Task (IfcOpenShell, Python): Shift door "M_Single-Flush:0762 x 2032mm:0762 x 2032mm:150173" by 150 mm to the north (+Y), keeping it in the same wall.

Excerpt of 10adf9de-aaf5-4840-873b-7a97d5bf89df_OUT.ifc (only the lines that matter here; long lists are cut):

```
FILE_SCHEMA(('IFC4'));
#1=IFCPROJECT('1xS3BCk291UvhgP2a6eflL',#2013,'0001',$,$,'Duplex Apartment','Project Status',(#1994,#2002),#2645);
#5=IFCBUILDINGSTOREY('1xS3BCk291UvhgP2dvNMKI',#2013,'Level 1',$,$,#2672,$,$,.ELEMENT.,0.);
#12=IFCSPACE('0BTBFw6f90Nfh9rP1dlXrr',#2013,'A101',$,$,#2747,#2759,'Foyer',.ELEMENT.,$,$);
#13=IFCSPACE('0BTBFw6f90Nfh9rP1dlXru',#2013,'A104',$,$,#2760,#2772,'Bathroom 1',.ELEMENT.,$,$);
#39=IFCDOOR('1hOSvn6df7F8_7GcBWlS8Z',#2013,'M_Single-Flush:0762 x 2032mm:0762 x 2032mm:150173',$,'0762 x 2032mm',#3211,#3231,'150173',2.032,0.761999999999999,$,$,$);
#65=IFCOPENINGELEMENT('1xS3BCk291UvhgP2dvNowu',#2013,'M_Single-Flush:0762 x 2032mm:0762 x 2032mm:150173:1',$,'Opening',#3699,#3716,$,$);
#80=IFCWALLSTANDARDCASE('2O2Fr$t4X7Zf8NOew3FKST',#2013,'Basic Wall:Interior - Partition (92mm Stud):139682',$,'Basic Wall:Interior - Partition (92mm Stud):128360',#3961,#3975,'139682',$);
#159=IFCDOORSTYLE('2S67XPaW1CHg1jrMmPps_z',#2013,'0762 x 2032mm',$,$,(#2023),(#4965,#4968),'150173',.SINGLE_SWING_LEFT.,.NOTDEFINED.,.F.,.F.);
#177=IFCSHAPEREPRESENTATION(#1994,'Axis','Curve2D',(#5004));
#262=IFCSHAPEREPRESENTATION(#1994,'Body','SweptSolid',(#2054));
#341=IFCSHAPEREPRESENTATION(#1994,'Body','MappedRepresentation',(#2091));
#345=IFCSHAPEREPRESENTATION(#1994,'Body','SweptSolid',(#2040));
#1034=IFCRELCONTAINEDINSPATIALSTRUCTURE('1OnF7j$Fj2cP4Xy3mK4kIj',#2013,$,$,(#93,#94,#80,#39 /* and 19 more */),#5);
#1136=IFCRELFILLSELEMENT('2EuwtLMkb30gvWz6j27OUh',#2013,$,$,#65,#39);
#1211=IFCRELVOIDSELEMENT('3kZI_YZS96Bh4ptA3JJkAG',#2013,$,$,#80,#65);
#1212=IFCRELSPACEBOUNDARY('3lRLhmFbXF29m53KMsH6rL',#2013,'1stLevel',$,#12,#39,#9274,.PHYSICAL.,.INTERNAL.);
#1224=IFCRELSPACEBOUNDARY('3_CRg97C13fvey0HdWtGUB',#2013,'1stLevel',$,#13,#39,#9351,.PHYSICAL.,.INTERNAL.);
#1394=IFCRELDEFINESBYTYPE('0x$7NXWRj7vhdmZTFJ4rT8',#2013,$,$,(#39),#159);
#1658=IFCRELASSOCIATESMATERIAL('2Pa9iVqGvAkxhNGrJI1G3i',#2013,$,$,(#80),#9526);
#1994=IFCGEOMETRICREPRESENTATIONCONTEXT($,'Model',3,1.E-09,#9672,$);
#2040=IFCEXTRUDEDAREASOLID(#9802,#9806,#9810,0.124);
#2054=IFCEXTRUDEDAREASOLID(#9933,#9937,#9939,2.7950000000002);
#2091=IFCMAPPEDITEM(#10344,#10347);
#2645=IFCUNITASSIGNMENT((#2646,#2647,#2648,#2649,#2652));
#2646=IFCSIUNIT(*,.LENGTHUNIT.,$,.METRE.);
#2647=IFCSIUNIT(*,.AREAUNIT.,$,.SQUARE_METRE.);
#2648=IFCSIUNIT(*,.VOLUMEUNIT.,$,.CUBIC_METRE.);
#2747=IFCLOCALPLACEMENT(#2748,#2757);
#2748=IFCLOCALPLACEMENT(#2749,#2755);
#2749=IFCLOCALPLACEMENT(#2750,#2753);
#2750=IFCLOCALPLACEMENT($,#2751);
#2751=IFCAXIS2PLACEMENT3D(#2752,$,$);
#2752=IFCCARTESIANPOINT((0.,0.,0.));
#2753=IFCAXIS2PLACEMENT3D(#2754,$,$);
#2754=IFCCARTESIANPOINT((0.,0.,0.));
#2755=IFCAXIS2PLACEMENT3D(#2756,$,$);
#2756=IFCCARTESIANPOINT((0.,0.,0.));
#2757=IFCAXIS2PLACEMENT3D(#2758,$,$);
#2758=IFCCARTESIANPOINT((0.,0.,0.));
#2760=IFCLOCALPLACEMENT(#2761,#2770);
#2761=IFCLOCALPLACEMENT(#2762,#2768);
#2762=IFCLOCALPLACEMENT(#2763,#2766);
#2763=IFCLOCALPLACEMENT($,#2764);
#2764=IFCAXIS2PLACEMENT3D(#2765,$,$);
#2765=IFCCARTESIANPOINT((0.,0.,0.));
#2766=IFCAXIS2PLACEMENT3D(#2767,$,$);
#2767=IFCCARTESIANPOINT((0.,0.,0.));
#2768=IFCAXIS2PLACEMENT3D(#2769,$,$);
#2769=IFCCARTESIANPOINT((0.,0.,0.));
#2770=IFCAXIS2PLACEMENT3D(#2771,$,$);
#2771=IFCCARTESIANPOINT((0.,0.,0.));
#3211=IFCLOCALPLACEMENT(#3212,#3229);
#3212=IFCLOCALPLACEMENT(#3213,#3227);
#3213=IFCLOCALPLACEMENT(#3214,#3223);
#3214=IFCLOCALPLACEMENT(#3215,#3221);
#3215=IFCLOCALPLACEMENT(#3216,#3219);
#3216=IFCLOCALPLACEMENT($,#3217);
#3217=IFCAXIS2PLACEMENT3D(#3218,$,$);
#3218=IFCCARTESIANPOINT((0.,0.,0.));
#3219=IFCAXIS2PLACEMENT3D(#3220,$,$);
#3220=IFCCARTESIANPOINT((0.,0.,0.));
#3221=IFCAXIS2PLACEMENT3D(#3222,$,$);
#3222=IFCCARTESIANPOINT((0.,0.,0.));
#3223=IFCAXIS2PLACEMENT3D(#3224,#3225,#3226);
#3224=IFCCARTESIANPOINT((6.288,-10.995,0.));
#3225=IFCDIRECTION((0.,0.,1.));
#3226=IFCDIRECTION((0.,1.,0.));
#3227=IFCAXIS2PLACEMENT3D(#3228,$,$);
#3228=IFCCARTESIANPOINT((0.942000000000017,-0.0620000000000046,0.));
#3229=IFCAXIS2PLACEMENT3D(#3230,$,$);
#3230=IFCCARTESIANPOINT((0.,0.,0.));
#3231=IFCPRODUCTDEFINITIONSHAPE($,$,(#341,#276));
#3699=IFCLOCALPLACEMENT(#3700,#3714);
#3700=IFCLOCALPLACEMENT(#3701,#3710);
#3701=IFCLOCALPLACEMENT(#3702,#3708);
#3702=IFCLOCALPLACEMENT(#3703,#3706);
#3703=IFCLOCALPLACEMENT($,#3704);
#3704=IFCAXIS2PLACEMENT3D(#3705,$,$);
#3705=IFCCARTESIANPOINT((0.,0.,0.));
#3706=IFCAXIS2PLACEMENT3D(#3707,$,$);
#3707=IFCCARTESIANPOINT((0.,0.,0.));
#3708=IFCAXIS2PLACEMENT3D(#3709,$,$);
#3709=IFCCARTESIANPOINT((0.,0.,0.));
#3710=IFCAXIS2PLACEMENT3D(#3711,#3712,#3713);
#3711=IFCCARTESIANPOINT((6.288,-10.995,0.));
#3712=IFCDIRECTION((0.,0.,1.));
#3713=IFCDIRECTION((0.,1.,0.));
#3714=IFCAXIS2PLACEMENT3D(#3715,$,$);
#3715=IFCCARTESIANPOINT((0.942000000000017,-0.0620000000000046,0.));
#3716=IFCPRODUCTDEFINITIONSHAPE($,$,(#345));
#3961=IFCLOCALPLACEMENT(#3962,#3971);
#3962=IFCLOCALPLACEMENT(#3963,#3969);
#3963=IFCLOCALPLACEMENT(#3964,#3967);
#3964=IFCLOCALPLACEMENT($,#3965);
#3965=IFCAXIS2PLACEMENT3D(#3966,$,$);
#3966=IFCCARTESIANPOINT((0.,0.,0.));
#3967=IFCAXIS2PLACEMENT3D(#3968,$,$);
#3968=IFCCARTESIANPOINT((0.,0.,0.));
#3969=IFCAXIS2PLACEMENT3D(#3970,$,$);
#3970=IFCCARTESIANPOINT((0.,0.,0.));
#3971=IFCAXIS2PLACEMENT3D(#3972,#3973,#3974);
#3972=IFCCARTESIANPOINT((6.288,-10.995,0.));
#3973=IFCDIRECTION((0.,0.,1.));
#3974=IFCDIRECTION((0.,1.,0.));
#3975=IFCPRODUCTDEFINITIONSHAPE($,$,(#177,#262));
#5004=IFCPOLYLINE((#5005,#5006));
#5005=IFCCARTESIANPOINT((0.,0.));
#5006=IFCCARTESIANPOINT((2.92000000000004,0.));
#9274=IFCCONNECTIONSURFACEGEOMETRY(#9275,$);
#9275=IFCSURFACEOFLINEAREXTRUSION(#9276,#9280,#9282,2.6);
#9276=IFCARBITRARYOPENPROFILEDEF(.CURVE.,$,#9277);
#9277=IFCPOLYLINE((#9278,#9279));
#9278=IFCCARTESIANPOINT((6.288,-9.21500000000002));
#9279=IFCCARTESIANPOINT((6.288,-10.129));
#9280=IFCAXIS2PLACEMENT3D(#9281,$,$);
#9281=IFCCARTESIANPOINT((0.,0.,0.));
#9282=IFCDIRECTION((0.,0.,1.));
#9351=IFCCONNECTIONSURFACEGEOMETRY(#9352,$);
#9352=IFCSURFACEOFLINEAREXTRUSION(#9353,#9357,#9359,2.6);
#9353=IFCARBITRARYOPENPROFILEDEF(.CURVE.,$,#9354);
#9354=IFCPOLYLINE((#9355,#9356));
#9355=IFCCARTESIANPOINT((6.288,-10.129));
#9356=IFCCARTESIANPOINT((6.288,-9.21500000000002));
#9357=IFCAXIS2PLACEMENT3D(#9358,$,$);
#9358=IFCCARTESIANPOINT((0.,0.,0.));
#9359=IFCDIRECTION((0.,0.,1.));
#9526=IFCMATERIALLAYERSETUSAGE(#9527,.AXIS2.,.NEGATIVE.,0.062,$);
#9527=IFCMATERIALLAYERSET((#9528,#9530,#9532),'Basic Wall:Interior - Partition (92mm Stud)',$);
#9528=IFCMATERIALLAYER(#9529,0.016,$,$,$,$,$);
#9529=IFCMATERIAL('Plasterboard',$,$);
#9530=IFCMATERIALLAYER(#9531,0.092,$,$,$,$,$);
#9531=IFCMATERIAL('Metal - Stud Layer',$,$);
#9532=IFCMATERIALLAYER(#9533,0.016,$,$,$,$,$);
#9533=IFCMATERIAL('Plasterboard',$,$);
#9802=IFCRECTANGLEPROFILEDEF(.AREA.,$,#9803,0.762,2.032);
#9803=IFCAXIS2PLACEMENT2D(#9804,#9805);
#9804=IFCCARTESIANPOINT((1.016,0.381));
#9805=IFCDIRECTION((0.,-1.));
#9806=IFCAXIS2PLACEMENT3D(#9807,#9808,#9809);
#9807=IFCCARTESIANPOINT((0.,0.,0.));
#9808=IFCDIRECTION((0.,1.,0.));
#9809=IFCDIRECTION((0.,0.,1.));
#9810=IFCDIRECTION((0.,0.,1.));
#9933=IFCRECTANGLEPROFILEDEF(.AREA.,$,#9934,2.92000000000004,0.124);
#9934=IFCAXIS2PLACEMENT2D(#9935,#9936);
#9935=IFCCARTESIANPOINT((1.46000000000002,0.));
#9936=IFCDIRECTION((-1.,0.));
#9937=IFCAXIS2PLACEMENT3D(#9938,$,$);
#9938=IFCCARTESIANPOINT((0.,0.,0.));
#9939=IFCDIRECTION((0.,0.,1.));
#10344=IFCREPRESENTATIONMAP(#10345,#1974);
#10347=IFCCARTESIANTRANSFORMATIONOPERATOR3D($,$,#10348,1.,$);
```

```python
import numpy as np
import ifcopenshell
import ifcopenshell.api.geometry
import ifcopenshell.util.placement
import ifcopenshell.util.unit

model = ifcopenshell.open("10adf9de-aaf5-4840-873b-7a97d5bf89df_OUT.ifc")
unit_scale = ifcopenshell.util.unit.calculate_unit_scale(model)

door = model.by_id(39)
opening = door.FillsVoids[0].RelatingOpeningElement
wall = opening.VoidsElements[0].RelatingBuildingElement

wall_matrix = ifcopenshell.util.placement.get_local_placement(wall.ObjectPlacement)
shift = wall_matrix[:3, 0] * 0.15 / unit_scale
before = ifcopenshell.util.placement.get_local_placement(door.ObjectPlacement)[:3, 3].copy()

# The door is not placed relative to its opening, so move both.
for product in (opening, door):
    matrix = ifcopenshell.util.placement.get_local_placement(product.ObjectPlacement)
    matrix[:3, 3] += shift
    ifcopenshell.api.geometry.edit_object_placement(model, product=product, matrix=matrix, is_si=False)

# Space boundary surfaces are stored in each space's coordinates; move them too.
for rel in door.ProvidesBoundaries:
    if not rel.ConnectionGeometry:
        continue
    surface = rel.ConnectionGeometry.SurfaceOnRelatingElement
    space_matrix = ifcopenshell.util.placement.get_local_placement(rel.RelatingSpace.ObjectPlacement)
    point = np.array(surface.Position.Location.Coordinates) + space_matrix[:3, :3].T @ shift
    surface.Position = model.createIfcAxis2Placement3D(
        model.createIfcCartesianPoint(point.tolist()), surface.Position.Axis, surface.Position.RefDirection
    )

after = ifcopenshell.util.placement.get_local_placement(door.ObjectPlacement)[:3, 3]
print("door moved by", (after - before).round(3) + 0.0)

model.write("10adf9de-aaf5-4840-873b-7a97d5bf89df_OUT_updated.ifc")
```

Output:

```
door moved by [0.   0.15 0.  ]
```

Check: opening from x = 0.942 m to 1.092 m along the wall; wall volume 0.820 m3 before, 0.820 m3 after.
